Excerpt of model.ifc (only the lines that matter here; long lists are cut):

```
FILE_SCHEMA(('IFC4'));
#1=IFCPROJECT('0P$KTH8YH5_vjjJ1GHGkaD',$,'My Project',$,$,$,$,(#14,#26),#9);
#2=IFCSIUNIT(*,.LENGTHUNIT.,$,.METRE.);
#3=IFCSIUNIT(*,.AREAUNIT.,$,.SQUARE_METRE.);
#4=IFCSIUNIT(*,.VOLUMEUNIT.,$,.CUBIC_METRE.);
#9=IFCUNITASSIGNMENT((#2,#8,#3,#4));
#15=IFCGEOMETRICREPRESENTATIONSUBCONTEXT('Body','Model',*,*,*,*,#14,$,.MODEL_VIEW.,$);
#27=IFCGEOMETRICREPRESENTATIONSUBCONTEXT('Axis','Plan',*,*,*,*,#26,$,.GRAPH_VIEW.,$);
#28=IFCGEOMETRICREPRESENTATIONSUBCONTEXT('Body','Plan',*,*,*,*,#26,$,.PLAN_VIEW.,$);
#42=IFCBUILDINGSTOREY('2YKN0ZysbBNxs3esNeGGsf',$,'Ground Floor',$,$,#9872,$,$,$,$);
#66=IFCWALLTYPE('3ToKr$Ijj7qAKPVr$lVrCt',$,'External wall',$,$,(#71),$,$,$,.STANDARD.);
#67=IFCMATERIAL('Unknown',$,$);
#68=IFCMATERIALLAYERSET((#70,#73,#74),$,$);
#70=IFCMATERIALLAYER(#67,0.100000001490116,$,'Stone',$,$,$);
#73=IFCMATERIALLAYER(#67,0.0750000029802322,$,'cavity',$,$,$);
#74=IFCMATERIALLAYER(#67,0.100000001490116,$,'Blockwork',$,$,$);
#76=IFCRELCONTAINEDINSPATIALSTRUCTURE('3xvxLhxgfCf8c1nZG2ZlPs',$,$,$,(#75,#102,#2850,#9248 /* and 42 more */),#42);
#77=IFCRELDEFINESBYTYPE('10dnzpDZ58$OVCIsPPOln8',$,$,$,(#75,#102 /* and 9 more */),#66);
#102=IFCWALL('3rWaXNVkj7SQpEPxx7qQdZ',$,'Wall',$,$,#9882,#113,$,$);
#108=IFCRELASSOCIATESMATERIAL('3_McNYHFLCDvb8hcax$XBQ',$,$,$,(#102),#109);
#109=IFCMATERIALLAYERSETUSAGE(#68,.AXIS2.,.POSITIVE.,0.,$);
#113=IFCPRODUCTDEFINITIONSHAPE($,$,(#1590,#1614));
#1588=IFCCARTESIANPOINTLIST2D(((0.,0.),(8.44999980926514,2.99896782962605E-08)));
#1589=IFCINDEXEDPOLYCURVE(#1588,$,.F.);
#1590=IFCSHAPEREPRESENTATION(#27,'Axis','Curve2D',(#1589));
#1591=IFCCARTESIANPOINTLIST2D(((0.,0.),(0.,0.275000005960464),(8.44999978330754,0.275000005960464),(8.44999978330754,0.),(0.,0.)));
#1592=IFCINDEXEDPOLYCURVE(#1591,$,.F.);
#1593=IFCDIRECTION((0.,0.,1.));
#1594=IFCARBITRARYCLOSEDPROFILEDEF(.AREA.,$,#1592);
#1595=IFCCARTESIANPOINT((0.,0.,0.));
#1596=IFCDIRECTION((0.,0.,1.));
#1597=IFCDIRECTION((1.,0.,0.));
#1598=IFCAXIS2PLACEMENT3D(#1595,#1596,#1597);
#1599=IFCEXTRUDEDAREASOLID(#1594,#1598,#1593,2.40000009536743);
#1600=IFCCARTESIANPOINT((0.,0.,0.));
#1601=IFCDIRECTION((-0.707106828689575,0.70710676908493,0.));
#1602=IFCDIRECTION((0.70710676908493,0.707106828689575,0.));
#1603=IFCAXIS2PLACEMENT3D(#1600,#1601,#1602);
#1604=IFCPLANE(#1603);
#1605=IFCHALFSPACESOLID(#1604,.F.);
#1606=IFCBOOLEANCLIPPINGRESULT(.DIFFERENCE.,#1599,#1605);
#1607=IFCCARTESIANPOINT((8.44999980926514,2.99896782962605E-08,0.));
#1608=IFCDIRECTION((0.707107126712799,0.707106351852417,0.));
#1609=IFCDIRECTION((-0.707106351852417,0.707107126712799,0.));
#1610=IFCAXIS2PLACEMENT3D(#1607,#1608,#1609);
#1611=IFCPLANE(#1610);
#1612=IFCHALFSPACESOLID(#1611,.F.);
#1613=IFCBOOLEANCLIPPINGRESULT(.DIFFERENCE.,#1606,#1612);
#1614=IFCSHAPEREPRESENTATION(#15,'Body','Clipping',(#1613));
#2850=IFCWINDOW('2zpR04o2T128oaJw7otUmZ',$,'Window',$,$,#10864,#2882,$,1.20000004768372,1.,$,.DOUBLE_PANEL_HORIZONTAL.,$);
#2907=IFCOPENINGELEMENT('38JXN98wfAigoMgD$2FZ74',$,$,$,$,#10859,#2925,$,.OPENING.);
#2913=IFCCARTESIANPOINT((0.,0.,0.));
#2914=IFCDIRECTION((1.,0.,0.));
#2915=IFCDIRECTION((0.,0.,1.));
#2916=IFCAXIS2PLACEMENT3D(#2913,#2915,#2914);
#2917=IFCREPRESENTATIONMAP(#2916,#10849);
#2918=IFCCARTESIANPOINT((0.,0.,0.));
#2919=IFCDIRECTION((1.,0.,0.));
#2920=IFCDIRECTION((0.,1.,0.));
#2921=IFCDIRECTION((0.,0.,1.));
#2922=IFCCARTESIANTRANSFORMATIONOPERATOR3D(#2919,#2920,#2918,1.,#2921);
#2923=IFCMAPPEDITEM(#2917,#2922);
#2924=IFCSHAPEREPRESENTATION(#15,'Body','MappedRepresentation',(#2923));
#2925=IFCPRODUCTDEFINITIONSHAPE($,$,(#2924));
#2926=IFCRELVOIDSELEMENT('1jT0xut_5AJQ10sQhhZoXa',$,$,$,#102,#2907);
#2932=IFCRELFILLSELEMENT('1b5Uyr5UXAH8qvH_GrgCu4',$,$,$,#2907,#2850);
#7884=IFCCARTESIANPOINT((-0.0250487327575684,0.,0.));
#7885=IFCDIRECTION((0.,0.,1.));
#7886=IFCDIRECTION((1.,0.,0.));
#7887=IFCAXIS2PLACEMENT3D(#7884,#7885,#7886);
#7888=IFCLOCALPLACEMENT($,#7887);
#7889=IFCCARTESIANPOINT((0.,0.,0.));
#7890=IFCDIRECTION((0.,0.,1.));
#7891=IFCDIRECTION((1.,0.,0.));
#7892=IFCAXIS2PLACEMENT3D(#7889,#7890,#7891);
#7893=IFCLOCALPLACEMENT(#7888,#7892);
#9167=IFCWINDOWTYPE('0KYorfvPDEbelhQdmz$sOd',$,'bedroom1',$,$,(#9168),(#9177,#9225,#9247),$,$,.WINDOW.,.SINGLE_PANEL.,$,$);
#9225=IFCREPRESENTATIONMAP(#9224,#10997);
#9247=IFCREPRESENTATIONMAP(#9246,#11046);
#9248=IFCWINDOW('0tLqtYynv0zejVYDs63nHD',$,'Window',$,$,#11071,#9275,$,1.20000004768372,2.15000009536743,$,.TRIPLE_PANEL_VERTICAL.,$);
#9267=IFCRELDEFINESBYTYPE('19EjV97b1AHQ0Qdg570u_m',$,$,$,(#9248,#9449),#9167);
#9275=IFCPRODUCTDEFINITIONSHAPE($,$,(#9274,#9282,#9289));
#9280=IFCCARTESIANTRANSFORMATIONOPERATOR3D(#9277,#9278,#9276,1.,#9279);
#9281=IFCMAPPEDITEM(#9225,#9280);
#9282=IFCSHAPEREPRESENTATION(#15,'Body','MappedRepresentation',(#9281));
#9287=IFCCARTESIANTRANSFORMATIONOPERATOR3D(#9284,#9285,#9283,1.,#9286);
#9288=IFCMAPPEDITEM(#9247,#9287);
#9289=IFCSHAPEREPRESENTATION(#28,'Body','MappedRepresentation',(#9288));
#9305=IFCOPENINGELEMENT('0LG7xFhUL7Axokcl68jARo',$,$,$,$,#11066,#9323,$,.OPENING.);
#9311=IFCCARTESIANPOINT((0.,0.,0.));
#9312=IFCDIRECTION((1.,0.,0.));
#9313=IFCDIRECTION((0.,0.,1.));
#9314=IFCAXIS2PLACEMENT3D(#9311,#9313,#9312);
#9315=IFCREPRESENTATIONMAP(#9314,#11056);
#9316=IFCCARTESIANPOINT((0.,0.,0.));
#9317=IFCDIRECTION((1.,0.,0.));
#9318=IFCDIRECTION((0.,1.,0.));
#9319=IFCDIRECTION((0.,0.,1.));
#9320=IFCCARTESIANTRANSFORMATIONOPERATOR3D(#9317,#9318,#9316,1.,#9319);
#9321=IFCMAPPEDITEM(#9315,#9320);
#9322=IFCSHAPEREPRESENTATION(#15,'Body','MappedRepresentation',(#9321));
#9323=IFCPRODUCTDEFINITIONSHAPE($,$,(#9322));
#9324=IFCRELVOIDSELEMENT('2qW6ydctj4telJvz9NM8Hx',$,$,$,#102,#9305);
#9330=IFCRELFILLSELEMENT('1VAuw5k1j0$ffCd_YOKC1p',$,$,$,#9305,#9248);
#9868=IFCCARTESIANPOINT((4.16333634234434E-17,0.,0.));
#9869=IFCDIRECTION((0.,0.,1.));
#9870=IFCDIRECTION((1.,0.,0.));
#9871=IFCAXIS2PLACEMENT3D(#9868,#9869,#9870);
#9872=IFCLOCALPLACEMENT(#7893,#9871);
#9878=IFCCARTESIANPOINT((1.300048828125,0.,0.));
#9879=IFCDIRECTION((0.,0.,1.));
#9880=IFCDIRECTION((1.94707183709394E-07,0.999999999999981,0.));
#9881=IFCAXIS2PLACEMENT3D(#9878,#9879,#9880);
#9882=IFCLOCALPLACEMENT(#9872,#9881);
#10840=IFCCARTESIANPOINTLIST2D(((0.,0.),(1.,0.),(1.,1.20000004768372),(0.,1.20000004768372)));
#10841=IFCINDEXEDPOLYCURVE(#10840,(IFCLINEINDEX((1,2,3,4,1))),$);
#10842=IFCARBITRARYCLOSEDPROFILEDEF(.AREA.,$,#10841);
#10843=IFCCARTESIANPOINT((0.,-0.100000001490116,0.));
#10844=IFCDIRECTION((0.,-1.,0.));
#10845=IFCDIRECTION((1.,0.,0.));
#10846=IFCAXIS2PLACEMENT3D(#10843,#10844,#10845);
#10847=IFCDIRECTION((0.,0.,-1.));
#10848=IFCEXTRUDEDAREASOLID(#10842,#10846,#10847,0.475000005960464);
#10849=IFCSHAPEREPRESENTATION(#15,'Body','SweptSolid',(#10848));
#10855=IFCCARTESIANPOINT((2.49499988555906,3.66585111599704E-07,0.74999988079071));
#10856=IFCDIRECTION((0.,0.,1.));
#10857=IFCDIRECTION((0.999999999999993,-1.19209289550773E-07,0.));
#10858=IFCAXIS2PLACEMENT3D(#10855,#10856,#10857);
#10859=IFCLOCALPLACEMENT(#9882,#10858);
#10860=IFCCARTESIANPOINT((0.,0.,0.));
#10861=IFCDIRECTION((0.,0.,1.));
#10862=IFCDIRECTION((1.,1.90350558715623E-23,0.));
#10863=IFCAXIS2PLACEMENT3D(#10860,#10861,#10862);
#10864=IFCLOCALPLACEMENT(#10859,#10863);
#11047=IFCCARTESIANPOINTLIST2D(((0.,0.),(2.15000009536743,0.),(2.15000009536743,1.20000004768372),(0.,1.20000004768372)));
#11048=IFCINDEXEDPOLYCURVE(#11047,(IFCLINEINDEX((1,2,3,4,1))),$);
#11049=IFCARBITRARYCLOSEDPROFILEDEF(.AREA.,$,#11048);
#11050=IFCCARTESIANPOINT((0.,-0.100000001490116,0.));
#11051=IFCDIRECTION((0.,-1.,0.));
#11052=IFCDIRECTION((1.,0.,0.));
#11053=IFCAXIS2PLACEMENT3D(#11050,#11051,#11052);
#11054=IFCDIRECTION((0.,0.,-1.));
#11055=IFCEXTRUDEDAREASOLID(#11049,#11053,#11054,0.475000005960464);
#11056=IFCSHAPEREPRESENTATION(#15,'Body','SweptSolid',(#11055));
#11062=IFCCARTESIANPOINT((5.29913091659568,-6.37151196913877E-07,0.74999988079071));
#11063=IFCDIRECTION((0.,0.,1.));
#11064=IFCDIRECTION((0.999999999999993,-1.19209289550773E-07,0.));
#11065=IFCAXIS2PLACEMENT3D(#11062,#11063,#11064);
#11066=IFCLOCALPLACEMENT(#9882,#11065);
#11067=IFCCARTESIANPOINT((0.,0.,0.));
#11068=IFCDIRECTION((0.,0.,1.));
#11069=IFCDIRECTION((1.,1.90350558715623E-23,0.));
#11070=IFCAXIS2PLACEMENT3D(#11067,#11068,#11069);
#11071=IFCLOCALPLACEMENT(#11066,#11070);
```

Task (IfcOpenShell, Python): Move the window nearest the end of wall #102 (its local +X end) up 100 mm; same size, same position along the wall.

```python
import numpy as np
import ifcopenshell
import ifcopenshell.api.geometry
import ifcopenshell.util.placement
import ifcopenshell.util.unit

model = ifcopenshell.open("model.ifc")
unit_scale = ifcopenshell.util.unit.calculate_unit_scale(model)

window = model.by_guid("0tLqtYynv0zejVYDs63nHD")
opening = window.FillsVoids[0].RelatingOpeningElement
dz = 0.1

shift = np.array([0.0, 0.0, dz])
# The window is placed relative to its opening, so it follows when the opening moves.
matrix = ifcopenshell.util.placement.get_local_placement(opening.ObjectPlacement)
matrix[:3, 3] += shift
ifcopenshell.api.geometry.edit_object_placement(
    model, product=opening, matrix=matrix, is_si=False, should_transform_children=True
)

print(f"moved by {dz * unit_scale:+.3f} m")

model.write("model_v2.ifc")
```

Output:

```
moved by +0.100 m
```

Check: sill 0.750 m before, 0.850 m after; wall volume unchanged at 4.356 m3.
